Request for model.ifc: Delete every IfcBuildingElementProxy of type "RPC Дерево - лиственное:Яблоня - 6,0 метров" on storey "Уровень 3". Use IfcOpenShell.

First a look at what the model holds.

```python
import ifcopenshell
import ifcopenshell.util.element

model = ifcopenshell.open("model.ifc")
print(model.schema)
storey = next(s for s in model.by_type("IfcBuildingStorey") if s.Name == "Уровень 3")
proxies = [e for e in ifcopenshell.util.element.get_decomposition(storey) if e.is_a("IfcBuildingElementProxy")]
seen = {}
for e in proxies:
    element_type = ifcopenshell.util.element.get_type(e)
    name = element_type.Name if element_type not in (None, e) else None
    seen[name] = seen.get(name, 0) + 1
for name, count in sorted(seen.items(), key=str):
    print(count, "x", name)
```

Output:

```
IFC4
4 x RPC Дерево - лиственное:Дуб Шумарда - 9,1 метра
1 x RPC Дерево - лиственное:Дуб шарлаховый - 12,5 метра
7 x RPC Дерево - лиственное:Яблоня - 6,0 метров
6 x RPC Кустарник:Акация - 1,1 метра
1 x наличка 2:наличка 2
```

```python
import ifcopenshell
import ifcopenshell.api.root
import ifcopenshell.util.element

model = ifcopenshell.open("model.ifc")

storey = next(s for s in model.by_type("IfcBuildingStorey") if s.Name == "Уровень 3")
proxies = [e for e in ifcopenshell.util.element.get_decomposition(storey) if e.is_a("IfcBuildingElementProxy")]
targets = [e for e in proxies if (t := ifcopenshell.util.element.get_type(e)) not in (None, e) and t.Name == "RPC Дерево - лиственное:Яблоня - 6,0 метров"]

for e in targets:
    ifcopenshell.api.root.remove_product(model, product=e)
print(len(targets), "removed")

model.write("model_rev.ifc")
```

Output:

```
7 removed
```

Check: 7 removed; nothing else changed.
